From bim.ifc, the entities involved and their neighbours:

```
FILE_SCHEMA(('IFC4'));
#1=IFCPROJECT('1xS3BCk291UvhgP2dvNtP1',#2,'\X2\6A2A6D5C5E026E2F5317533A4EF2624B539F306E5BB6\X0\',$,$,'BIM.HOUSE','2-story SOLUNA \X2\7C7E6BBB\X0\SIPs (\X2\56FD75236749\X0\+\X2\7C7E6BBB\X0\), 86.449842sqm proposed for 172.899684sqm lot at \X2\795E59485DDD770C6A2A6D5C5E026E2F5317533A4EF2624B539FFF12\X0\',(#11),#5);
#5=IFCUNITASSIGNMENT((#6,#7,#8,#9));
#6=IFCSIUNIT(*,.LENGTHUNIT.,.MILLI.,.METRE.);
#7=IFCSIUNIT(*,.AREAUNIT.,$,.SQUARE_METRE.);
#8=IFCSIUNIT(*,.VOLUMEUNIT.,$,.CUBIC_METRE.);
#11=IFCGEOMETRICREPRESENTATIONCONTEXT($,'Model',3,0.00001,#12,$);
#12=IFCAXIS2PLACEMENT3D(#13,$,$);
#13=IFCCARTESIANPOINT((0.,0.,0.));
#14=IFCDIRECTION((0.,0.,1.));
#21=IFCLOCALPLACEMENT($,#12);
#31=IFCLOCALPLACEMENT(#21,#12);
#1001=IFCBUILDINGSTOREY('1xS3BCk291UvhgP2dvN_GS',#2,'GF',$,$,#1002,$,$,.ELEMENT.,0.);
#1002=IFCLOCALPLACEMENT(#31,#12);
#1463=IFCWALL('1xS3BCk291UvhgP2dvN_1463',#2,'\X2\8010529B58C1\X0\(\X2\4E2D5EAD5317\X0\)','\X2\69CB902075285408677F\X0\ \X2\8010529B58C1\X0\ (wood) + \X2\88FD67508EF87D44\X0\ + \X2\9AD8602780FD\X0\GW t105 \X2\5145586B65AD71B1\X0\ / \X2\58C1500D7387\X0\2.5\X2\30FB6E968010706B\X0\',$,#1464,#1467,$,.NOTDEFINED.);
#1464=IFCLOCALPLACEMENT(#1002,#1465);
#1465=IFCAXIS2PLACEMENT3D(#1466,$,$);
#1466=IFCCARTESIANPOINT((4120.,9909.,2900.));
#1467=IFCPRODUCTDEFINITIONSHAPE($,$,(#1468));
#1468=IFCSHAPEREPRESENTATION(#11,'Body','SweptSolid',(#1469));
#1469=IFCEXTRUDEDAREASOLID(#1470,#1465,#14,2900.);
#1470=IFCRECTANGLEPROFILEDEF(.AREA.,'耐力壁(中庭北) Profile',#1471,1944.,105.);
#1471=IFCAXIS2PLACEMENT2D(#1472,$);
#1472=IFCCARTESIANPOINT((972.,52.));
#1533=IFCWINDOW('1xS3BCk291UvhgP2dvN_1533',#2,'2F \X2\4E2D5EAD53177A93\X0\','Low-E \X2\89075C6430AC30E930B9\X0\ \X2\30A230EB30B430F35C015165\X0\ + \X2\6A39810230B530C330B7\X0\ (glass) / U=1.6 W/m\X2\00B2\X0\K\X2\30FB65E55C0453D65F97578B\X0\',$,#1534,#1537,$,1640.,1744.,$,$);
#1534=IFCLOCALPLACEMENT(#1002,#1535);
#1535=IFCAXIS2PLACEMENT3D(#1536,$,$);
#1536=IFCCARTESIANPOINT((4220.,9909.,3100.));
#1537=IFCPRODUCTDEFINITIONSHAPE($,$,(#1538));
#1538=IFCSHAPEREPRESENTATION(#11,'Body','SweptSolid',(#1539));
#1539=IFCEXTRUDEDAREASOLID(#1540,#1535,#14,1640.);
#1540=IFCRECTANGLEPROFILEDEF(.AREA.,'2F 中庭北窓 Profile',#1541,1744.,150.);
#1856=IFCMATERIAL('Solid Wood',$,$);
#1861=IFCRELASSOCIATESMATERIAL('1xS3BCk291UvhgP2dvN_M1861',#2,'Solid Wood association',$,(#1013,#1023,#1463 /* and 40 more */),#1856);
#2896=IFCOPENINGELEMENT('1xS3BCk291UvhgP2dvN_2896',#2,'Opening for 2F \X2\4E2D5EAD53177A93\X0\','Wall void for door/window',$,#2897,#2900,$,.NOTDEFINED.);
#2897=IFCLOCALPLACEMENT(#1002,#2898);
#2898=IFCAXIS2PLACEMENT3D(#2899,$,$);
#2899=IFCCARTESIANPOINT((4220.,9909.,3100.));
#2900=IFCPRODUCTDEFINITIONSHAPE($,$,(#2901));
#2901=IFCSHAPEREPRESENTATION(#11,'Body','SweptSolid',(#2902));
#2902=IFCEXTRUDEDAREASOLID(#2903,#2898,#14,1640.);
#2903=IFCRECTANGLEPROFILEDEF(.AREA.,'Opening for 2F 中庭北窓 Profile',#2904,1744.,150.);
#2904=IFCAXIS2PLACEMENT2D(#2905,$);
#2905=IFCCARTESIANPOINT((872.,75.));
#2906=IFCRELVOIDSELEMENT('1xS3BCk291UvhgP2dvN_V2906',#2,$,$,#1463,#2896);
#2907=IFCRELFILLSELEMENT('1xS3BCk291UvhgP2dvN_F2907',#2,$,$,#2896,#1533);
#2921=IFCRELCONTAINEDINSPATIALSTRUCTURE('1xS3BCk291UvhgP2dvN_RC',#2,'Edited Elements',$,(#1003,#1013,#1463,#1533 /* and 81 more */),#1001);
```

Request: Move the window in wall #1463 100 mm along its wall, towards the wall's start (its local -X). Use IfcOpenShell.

```python
import ifcopenshell
import ifcopenshell.api.geometry
import ifcopenshell.util.placement
import ifcopenshell.util.unit

model = ifcopenshell.open("bim.ifc")
unit_scale = ifcopenshell.util.unit.calculate_unit_scale(model)

window = model.by_guid("1xS3BCk291UvhgP2dvN_1533")
opening = window.FillsVoids[0].RelatingOpeningElement
wall = opening.VoidsElements[0].RelatingBuildingElement

wall_matrix = ifcopenshell.util.placement.get_local_placement(wall.ObjectPlacement)
shift = wall_matrix[:3, 0] * -0.1 / unit_scale
before = ifcopenshell.util.placement.get_local_placement(window.ObjectPlacement)[:3, 3].copy()

# The window is not placed relative to its opening, so move both.
for product in (opening, window):
    matrix = ifcopenshell.util.placement.get_local_placement(product.ObjectPlacement)
    matrix[:3, 3] += shift
    ifcopenshell.api.geometry.edit_object_placement(model, product=product, matrix=matrix, is_si=False)

after = ifcopenshell.util.placement.get_local_placement(window.ObjectPlacement)[:3, 3]
print("window moved by", (after - before).round(3) + 0.0)

model.write("bim_v2.ifc")
```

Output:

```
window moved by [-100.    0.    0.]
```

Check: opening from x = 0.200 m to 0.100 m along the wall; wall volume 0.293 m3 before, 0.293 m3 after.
